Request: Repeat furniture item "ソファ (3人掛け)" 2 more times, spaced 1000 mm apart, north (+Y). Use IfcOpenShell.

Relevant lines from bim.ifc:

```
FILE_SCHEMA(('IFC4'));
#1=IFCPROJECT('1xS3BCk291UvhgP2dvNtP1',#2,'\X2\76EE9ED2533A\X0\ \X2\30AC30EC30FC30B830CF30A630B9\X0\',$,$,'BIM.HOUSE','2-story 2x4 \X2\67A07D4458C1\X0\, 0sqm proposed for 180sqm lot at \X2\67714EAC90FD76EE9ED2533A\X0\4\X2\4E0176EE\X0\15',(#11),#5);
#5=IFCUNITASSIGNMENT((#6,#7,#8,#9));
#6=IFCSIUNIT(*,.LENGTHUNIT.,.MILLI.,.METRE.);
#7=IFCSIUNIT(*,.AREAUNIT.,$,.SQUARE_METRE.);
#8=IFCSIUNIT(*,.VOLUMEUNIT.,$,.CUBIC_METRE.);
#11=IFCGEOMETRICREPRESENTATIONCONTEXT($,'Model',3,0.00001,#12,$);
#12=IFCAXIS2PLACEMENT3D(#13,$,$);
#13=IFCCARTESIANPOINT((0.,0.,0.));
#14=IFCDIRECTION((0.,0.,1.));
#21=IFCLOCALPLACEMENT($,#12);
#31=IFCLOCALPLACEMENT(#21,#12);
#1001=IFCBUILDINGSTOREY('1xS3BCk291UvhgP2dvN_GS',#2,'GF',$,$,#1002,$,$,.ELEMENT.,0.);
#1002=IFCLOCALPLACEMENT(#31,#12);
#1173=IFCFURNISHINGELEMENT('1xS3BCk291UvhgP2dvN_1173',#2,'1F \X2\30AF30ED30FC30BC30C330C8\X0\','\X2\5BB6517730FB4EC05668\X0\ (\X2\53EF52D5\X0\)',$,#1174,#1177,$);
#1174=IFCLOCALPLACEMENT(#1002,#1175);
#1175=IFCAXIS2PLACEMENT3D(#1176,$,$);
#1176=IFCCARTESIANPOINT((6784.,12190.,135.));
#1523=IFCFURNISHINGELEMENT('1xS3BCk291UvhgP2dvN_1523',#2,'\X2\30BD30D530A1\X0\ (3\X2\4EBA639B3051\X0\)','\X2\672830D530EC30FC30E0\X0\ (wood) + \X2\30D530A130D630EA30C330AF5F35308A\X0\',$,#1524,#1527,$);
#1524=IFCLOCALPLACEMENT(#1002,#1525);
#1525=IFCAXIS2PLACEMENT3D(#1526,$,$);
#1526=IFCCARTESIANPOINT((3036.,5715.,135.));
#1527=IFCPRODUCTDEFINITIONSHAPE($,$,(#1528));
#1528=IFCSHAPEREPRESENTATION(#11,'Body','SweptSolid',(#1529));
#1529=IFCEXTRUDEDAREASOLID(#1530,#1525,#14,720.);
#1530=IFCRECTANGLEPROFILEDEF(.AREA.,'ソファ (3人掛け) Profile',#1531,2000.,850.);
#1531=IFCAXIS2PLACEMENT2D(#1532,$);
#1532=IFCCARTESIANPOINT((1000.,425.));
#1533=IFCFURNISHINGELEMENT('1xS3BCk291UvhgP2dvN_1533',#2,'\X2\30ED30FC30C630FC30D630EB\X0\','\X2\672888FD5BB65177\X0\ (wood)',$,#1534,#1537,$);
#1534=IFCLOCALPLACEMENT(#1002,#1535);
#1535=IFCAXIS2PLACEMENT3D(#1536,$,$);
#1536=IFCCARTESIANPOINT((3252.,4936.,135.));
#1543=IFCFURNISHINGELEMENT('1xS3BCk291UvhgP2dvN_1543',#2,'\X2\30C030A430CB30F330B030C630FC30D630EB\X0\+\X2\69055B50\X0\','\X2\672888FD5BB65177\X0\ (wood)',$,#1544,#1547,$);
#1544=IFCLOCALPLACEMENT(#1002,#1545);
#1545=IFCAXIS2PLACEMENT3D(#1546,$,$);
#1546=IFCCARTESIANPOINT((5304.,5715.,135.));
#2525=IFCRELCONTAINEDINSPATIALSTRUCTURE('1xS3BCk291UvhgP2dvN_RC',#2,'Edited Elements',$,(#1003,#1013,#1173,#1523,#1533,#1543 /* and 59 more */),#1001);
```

```python
import numpy as np
import ifcopenshell
import ifcopenshell.api.geometry
import ifcopenshell.api.root
import ifcopenshell.util.element
import ifcopenshell.util.placement

model = ifcopenshell.open("bim.ifc")


def reuse_history(source, copy):
    """copy_class also copies each property set's owner history, people and application; keep the originals."""
    for rel in copy.IsDefinedBy:
        if rel.is_a("IfcRelDefinesByProperties") and (history := rel.RelatingPropertyDefinition.OwnerHistory):
            rel.RelatingPropertyDefinition.OwnerHistory = source.OwnerHistory
            ifcopenshell.util.element.remove_deep2(model, history)


source = model.by_guid("1xS3BCk291UvhgP2dvN_1523")
base = ifcopenshell.util.placement.get_local_placement(source.ObjectPlacement)
step = np.array([0.0, 1.0, 0.0]) * 1000.0

for i in range(1, 3):
    copy = ifcopenshell.api.root.copy_class(model, product=source)
    copy.Representation = ifcopenshell.util.element.copy_deep(
        model, source.Representation, exclude=["IfcGeometricRepresentationContext", "IfcRepresentationMap"]
    )
    reuse_history(source, copy)
    matrix = base.copy()
    matrix[:3, 3] += i * step
    print("added at", matrix[:3, 3].round(3) + 0.0)
    ifcopenshell.api.geometry.edit_object_placement(model, product=copy, matrix=matrix, is_si=False)

model.write("bim-out.ifc")
```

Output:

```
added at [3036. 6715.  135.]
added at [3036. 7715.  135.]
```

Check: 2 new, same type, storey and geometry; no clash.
